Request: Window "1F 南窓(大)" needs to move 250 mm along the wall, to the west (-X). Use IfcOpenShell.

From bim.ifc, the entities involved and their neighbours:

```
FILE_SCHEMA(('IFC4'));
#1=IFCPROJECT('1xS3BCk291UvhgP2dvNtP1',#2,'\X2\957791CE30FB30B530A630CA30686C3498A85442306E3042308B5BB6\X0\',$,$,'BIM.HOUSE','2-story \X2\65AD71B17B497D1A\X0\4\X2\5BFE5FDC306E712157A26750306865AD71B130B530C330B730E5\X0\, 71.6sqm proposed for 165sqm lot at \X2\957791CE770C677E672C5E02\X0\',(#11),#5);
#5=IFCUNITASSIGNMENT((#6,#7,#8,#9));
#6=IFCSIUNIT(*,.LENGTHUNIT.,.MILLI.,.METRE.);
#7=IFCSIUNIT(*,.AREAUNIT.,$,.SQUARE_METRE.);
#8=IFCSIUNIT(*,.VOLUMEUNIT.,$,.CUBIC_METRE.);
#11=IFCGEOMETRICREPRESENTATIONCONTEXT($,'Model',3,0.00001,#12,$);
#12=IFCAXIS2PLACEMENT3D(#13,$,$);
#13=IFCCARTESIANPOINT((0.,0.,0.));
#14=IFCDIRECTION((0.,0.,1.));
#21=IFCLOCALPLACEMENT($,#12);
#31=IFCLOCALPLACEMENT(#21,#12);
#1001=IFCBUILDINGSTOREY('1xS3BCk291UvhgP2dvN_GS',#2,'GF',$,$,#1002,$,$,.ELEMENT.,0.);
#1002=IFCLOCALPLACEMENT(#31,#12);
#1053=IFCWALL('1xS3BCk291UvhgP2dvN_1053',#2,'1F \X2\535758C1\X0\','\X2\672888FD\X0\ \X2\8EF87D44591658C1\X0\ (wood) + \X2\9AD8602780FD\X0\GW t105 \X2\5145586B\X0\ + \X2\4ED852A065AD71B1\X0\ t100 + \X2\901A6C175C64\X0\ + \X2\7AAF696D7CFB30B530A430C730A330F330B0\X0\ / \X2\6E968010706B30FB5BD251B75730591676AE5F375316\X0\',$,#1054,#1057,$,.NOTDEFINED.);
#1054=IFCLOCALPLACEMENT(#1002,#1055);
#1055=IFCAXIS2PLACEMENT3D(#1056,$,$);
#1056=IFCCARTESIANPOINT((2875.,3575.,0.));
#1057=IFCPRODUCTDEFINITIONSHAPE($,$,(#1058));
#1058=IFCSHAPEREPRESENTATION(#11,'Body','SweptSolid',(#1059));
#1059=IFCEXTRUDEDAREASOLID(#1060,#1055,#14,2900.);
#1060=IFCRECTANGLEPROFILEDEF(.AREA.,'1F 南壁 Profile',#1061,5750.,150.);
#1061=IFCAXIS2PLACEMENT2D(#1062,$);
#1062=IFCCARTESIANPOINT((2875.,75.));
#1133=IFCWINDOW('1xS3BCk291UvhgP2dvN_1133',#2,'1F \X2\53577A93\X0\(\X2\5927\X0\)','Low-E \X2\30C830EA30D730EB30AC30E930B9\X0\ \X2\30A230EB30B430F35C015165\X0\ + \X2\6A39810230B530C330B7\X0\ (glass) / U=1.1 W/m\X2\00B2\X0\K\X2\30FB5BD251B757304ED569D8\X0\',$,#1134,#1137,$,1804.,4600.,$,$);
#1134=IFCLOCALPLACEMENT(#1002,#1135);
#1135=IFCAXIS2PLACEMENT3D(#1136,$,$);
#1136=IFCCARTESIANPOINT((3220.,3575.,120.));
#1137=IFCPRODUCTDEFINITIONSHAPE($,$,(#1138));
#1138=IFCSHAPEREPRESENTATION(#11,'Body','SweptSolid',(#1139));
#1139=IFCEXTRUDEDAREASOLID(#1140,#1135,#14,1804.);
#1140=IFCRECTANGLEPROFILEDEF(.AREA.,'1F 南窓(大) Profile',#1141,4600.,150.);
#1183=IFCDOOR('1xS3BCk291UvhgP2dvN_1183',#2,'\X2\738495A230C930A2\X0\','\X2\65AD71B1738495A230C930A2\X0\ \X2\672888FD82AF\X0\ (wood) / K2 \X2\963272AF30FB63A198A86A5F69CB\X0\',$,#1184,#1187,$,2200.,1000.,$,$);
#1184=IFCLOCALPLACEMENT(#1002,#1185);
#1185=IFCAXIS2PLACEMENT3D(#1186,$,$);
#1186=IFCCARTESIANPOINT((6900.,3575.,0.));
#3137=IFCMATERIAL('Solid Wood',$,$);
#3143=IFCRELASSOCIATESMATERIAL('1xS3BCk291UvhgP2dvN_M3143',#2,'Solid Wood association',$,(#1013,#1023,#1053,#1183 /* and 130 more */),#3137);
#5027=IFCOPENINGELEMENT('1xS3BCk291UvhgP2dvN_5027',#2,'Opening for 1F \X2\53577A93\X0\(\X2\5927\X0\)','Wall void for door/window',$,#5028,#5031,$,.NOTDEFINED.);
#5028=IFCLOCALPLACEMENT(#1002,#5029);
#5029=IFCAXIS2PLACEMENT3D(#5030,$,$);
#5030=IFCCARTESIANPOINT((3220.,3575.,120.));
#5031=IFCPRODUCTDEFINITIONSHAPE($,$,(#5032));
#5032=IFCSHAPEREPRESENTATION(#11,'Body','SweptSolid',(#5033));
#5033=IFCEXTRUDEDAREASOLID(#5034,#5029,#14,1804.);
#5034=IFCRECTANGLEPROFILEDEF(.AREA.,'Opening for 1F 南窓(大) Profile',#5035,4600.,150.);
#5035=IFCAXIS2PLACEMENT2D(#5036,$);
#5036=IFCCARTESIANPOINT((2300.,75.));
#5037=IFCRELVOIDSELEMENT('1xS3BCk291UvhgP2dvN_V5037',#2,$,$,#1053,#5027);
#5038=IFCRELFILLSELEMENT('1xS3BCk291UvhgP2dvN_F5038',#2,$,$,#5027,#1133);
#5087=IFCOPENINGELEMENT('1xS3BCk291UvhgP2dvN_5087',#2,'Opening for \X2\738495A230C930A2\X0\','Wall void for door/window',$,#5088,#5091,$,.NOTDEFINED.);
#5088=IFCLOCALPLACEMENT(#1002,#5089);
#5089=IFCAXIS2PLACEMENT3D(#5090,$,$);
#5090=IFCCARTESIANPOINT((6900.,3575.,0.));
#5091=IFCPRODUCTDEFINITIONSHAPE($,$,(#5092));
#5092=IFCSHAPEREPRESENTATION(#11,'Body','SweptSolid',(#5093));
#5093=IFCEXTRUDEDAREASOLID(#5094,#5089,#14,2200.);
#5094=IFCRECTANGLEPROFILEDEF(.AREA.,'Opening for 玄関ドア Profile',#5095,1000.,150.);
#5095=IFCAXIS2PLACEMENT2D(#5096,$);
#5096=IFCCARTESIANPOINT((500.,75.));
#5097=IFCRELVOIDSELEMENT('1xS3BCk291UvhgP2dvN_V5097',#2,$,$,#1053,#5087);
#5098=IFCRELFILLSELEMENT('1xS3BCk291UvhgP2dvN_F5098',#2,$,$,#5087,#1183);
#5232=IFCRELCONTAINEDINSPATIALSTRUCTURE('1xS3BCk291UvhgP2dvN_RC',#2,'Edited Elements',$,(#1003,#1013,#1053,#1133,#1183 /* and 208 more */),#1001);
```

```python
import ifcopenshell
import ifcopenshell.api.geometry
import ifcopenshell.util.placement

model = ifcopenshell.open("bim.ifc")

window = model.by_guid("1xS3BCk291UvhgP2dvN_1133")
opening = window.FillsVoids[0].RelatingOpeningElement
wall = opening.VoidsElements[0].RelatingBuildingElement

wall_matrix = ifcopenshell.util.placement.get_local_placement(wall.ObjectPlacement)
shift = wall_matrix[:3, 0] * -250.0
before = ifcopenshell.util.placement.get_local_placement(window.ObjectPlacement)[:3, 3].copy()

# The window is not placed relative to its opening, so move both.
for product in (opening, window):
    matrix = ifcopenshell.util.placement.get_local_placement(product.ObjectPlacement)
    matrix[:3, 3] += shift
    ifcopenshell.api.geometry.edit_object_placement(model, product=product, matrix=matrix, is_si=False)

after = ifcopenshell.util.placement.get_local_placement(window.ObjectPlacement)[:3, 3]
print("window moved by", (after - before).round(3) + 0.0)

model.write("bim_updated.ifc")
```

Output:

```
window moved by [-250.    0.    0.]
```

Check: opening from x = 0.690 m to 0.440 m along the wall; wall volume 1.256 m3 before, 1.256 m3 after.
